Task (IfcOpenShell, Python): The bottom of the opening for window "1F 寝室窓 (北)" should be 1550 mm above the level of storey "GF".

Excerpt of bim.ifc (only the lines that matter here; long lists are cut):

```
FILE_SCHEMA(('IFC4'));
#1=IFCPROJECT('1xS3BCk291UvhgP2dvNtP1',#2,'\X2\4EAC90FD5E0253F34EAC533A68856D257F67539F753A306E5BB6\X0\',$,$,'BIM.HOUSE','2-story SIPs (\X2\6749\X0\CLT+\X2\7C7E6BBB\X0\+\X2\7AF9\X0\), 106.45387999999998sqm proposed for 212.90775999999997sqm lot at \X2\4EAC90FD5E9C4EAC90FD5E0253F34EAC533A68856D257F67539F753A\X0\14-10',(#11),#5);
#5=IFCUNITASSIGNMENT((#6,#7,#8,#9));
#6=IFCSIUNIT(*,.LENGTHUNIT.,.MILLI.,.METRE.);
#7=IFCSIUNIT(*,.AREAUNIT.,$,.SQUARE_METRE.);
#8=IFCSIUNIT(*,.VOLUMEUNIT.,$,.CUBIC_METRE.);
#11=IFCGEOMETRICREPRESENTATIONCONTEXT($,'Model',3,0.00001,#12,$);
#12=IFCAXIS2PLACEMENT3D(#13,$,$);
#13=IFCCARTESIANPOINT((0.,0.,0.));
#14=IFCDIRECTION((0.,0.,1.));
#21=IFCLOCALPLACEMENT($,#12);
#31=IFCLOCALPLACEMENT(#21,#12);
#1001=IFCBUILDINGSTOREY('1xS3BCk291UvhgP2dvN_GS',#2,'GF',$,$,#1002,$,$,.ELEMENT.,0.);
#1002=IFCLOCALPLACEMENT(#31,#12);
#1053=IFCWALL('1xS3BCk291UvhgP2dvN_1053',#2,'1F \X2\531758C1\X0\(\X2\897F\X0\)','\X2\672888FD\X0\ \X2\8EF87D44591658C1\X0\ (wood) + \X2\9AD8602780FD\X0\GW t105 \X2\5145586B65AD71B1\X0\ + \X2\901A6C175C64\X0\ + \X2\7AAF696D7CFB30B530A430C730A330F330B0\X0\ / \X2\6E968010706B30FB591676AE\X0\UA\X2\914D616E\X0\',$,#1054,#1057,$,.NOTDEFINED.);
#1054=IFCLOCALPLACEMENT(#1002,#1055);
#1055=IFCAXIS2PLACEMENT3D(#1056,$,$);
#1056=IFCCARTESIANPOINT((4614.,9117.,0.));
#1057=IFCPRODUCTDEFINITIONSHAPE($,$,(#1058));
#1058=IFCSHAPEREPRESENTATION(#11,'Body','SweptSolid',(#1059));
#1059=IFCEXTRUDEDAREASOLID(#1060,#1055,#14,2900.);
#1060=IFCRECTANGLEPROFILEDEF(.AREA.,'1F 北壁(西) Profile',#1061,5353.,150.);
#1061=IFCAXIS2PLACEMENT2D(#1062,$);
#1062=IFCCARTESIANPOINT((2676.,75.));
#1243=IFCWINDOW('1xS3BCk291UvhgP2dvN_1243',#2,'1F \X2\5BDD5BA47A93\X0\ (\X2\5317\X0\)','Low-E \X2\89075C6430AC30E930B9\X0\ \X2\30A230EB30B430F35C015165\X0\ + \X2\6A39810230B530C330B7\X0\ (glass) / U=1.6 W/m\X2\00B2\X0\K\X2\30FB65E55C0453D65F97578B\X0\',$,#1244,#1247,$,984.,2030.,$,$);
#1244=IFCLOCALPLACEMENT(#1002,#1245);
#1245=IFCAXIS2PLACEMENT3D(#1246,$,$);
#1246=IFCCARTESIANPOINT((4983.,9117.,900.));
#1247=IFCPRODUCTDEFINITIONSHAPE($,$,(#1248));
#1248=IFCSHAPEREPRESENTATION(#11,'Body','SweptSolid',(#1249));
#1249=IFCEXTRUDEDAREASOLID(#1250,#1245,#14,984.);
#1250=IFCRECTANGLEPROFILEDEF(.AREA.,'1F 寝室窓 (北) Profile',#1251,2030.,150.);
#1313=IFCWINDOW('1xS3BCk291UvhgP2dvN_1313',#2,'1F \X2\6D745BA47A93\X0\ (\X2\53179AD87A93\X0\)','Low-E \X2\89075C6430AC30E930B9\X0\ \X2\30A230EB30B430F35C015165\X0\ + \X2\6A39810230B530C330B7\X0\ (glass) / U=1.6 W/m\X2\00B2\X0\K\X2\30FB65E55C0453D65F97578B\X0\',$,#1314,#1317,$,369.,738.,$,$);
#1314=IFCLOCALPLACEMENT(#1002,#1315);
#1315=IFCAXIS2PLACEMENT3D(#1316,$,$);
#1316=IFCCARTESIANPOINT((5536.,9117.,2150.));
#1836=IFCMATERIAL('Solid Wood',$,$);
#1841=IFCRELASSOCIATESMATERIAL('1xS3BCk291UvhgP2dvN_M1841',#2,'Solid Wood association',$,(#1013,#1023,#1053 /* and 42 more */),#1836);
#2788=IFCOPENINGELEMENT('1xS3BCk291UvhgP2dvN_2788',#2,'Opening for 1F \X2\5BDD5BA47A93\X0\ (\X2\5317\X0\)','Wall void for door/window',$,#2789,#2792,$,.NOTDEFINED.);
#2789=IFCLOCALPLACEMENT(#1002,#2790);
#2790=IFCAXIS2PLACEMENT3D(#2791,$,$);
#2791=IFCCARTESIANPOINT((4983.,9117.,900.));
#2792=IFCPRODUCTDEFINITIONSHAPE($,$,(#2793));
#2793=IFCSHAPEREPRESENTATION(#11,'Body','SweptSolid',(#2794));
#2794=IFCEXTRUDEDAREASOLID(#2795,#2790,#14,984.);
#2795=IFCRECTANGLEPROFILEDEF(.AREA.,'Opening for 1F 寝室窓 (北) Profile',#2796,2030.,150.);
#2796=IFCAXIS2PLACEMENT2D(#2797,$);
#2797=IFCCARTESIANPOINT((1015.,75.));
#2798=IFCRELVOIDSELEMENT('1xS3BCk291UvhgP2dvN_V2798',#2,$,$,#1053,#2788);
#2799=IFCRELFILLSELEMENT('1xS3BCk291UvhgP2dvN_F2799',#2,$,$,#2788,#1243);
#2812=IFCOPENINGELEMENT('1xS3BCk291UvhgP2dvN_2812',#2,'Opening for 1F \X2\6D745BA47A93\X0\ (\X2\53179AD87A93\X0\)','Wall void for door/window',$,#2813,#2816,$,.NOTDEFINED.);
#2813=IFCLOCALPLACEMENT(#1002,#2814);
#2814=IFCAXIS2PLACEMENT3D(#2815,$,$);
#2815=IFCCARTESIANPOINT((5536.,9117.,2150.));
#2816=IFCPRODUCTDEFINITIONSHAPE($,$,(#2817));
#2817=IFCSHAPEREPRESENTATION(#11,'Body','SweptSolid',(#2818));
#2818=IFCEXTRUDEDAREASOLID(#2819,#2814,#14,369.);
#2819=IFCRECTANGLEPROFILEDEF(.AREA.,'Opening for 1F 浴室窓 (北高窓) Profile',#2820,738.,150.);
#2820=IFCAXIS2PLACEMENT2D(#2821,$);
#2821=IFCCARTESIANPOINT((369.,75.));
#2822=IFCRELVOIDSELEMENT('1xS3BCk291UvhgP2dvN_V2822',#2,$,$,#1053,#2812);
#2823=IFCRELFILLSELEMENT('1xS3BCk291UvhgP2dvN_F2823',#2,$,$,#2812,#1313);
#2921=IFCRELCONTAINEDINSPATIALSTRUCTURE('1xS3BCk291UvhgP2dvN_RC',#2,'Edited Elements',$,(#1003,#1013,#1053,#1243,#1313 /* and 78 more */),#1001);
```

```python
import numpy as np
import ifcopenshell
import ifcopenshell.api.geometry
import ifcopenshell.geom
import ifcopenshell.util.element
import ifcopenshell.util.placement
import ifcopenshell.util.shape
import ifcopenshell.util.unit

model = ifcopenshell.open("bim.ifc")
unit_scale = ifcopenshell.util.unit.calculate_unit_scale(model)

window = model.by_id(1243)
opening = window.FillsVoids[0].RelatingOpeningElement
storey = ifcopenshell.util.element.get_container(window, ifc_class="IfcBuildingStorey")
level = ifcopenshell.util.placement.get_local_placement(storey.ObjectPlacement)[2, 3]

# The opening's origin need not be at the sill, so measure its lowest point.
shape = ifcopenshell.geom.create_shape(ifcopenshell.geom.settings(), opening)
bottom = ifcopenshell.util.shape.get_shape_bottom_elevation(shape, shape.geometry) / unit_scale
dz = level + 1.55 / unit_scale - bottom

shift = np.array([0.0, 0.0, dz])
# The window is not placed relative to its opening, so move both.
for product in (opening, window):
    matrix = ifcopenshell.util.placement.get_local_placement(product.ObjectPlacement)
    matrix[:3, 3] += shift
    ifcopenshell.api.geometry.edit_object_placement(model, product=product, matrix=matrix, is_si=False)

print(f"moved by {dz * unit_scale:+.3f} m")

model.write("bim_v2.ifc")
```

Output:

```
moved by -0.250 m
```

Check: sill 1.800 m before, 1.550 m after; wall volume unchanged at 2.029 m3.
